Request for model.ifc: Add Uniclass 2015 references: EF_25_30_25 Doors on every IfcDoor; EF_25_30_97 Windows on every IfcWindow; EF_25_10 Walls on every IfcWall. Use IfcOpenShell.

First a look at what the model holds.

```python
import ifcopenshell

model = ifcopenshell.open("model.ifc")
print(model.schema)
print("classifications:", [c.Name for c in model.by_type("IfcClassification")])
for ifc_class in ("IfcDoor", "IfcRoof", "IfcStair", "IfcWall", "IfcWindow"):
    print(ifc_class, len(model.by_type(ifc_class)))
```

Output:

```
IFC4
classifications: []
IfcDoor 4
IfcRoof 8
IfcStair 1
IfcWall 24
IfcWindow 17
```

```python
import ifcopenshell
import ifcopenshell.api.classification

model = ifcopenshell.open("model.ifc")

system = ifcopenshell.api.classification.add_classification(model, classification="Uniclass 2015")

codes = {
    "IfcDoor": ("EF_25_30_25", "Doors"),
    "IfcWindow": ("EF_25_30_97", "Windows"),
    "IfcWall": ("EF_25_10", "Walls"),
}
for ifc_class, (code, name) in codes.items():
    products = model.by_type(ifc_class)
    ifcopenshell.api.classification.add_reference(
        model, products=products, classification=system, identification=code, name=name
    )
    print(code, len(products))

model.write("model-out.ifc")
```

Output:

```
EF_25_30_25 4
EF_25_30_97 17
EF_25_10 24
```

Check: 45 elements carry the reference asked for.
